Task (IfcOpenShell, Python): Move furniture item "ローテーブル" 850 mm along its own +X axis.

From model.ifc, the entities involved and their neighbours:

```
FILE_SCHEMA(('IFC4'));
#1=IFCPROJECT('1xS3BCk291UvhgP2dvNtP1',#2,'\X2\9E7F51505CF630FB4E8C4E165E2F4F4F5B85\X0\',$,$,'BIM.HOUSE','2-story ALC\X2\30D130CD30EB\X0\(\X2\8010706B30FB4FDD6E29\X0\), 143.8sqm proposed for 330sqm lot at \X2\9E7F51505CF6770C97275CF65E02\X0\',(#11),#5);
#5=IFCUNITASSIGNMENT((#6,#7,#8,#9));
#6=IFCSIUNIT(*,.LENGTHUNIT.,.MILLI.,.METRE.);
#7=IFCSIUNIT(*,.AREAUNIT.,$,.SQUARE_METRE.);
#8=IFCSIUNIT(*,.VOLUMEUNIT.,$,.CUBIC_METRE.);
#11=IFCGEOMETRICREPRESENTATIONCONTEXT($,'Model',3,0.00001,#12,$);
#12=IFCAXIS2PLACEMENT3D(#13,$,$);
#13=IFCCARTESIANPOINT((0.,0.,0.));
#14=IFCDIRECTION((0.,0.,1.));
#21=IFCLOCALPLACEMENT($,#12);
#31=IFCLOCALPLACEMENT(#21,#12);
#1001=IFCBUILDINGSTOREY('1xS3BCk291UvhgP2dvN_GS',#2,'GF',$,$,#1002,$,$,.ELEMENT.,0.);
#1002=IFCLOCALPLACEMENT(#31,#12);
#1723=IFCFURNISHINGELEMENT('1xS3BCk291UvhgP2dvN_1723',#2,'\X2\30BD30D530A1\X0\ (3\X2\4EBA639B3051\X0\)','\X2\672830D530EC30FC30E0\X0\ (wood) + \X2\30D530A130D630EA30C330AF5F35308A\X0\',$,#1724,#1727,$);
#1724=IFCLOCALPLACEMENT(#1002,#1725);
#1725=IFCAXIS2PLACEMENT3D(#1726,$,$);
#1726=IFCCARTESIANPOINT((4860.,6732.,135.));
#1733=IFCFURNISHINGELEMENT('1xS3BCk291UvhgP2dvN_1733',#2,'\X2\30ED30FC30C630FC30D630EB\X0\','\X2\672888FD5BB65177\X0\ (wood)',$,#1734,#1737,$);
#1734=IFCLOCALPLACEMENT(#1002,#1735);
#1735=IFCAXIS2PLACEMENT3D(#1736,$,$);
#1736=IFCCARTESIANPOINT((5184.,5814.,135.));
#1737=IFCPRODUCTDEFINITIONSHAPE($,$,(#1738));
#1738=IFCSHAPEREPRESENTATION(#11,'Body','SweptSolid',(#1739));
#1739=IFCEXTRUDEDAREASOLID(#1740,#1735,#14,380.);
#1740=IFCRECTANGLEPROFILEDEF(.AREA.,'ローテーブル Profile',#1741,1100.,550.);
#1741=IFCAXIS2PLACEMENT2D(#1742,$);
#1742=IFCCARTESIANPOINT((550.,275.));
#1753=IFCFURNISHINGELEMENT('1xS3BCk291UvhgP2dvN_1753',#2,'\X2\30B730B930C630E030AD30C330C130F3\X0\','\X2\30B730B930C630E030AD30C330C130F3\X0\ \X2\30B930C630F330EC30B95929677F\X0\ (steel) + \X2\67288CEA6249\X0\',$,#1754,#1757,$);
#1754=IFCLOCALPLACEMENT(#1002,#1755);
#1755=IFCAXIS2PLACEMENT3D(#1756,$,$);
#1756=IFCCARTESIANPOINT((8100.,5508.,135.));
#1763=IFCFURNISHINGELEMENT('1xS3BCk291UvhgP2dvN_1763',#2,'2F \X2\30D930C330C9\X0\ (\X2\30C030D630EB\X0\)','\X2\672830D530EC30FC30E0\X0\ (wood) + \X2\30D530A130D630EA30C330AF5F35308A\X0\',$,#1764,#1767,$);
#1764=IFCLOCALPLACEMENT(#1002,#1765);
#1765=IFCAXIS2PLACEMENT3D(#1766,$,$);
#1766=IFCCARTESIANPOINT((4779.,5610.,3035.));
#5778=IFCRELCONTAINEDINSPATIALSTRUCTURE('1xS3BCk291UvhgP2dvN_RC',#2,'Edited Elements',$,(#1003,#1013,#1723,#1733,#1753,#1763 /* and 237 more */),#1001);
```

```python
import ifcopenshell
import ifcopenshell.api.geometry
import ifcopenshell.util.placement

model = ifcopenshell.open("model.ifc")

item = model.by_id(1733)
matrix = ifcopenshell.util.placement.get_local_placement(item.ObjectPlacement)
matrix[:3, 3] += matrix[:3, 0] * 850.0
ifcopenshell.api.geometry.edit_object_placement(model, product=item, matrix=matrix, is_si=False)

print(ifcopenshell.util.placement.get_local_placement(item.ObjectPlacement).round(3) + 0.0)

model.write("model-out.ifc")
```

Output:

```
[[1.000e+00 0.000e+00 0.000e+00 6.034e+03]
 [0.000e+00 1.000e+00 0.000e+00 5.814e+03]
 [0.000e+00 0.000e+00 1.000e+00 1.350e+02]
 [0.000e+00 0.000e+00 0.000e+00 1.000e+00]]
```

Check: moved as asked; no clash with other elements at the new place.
